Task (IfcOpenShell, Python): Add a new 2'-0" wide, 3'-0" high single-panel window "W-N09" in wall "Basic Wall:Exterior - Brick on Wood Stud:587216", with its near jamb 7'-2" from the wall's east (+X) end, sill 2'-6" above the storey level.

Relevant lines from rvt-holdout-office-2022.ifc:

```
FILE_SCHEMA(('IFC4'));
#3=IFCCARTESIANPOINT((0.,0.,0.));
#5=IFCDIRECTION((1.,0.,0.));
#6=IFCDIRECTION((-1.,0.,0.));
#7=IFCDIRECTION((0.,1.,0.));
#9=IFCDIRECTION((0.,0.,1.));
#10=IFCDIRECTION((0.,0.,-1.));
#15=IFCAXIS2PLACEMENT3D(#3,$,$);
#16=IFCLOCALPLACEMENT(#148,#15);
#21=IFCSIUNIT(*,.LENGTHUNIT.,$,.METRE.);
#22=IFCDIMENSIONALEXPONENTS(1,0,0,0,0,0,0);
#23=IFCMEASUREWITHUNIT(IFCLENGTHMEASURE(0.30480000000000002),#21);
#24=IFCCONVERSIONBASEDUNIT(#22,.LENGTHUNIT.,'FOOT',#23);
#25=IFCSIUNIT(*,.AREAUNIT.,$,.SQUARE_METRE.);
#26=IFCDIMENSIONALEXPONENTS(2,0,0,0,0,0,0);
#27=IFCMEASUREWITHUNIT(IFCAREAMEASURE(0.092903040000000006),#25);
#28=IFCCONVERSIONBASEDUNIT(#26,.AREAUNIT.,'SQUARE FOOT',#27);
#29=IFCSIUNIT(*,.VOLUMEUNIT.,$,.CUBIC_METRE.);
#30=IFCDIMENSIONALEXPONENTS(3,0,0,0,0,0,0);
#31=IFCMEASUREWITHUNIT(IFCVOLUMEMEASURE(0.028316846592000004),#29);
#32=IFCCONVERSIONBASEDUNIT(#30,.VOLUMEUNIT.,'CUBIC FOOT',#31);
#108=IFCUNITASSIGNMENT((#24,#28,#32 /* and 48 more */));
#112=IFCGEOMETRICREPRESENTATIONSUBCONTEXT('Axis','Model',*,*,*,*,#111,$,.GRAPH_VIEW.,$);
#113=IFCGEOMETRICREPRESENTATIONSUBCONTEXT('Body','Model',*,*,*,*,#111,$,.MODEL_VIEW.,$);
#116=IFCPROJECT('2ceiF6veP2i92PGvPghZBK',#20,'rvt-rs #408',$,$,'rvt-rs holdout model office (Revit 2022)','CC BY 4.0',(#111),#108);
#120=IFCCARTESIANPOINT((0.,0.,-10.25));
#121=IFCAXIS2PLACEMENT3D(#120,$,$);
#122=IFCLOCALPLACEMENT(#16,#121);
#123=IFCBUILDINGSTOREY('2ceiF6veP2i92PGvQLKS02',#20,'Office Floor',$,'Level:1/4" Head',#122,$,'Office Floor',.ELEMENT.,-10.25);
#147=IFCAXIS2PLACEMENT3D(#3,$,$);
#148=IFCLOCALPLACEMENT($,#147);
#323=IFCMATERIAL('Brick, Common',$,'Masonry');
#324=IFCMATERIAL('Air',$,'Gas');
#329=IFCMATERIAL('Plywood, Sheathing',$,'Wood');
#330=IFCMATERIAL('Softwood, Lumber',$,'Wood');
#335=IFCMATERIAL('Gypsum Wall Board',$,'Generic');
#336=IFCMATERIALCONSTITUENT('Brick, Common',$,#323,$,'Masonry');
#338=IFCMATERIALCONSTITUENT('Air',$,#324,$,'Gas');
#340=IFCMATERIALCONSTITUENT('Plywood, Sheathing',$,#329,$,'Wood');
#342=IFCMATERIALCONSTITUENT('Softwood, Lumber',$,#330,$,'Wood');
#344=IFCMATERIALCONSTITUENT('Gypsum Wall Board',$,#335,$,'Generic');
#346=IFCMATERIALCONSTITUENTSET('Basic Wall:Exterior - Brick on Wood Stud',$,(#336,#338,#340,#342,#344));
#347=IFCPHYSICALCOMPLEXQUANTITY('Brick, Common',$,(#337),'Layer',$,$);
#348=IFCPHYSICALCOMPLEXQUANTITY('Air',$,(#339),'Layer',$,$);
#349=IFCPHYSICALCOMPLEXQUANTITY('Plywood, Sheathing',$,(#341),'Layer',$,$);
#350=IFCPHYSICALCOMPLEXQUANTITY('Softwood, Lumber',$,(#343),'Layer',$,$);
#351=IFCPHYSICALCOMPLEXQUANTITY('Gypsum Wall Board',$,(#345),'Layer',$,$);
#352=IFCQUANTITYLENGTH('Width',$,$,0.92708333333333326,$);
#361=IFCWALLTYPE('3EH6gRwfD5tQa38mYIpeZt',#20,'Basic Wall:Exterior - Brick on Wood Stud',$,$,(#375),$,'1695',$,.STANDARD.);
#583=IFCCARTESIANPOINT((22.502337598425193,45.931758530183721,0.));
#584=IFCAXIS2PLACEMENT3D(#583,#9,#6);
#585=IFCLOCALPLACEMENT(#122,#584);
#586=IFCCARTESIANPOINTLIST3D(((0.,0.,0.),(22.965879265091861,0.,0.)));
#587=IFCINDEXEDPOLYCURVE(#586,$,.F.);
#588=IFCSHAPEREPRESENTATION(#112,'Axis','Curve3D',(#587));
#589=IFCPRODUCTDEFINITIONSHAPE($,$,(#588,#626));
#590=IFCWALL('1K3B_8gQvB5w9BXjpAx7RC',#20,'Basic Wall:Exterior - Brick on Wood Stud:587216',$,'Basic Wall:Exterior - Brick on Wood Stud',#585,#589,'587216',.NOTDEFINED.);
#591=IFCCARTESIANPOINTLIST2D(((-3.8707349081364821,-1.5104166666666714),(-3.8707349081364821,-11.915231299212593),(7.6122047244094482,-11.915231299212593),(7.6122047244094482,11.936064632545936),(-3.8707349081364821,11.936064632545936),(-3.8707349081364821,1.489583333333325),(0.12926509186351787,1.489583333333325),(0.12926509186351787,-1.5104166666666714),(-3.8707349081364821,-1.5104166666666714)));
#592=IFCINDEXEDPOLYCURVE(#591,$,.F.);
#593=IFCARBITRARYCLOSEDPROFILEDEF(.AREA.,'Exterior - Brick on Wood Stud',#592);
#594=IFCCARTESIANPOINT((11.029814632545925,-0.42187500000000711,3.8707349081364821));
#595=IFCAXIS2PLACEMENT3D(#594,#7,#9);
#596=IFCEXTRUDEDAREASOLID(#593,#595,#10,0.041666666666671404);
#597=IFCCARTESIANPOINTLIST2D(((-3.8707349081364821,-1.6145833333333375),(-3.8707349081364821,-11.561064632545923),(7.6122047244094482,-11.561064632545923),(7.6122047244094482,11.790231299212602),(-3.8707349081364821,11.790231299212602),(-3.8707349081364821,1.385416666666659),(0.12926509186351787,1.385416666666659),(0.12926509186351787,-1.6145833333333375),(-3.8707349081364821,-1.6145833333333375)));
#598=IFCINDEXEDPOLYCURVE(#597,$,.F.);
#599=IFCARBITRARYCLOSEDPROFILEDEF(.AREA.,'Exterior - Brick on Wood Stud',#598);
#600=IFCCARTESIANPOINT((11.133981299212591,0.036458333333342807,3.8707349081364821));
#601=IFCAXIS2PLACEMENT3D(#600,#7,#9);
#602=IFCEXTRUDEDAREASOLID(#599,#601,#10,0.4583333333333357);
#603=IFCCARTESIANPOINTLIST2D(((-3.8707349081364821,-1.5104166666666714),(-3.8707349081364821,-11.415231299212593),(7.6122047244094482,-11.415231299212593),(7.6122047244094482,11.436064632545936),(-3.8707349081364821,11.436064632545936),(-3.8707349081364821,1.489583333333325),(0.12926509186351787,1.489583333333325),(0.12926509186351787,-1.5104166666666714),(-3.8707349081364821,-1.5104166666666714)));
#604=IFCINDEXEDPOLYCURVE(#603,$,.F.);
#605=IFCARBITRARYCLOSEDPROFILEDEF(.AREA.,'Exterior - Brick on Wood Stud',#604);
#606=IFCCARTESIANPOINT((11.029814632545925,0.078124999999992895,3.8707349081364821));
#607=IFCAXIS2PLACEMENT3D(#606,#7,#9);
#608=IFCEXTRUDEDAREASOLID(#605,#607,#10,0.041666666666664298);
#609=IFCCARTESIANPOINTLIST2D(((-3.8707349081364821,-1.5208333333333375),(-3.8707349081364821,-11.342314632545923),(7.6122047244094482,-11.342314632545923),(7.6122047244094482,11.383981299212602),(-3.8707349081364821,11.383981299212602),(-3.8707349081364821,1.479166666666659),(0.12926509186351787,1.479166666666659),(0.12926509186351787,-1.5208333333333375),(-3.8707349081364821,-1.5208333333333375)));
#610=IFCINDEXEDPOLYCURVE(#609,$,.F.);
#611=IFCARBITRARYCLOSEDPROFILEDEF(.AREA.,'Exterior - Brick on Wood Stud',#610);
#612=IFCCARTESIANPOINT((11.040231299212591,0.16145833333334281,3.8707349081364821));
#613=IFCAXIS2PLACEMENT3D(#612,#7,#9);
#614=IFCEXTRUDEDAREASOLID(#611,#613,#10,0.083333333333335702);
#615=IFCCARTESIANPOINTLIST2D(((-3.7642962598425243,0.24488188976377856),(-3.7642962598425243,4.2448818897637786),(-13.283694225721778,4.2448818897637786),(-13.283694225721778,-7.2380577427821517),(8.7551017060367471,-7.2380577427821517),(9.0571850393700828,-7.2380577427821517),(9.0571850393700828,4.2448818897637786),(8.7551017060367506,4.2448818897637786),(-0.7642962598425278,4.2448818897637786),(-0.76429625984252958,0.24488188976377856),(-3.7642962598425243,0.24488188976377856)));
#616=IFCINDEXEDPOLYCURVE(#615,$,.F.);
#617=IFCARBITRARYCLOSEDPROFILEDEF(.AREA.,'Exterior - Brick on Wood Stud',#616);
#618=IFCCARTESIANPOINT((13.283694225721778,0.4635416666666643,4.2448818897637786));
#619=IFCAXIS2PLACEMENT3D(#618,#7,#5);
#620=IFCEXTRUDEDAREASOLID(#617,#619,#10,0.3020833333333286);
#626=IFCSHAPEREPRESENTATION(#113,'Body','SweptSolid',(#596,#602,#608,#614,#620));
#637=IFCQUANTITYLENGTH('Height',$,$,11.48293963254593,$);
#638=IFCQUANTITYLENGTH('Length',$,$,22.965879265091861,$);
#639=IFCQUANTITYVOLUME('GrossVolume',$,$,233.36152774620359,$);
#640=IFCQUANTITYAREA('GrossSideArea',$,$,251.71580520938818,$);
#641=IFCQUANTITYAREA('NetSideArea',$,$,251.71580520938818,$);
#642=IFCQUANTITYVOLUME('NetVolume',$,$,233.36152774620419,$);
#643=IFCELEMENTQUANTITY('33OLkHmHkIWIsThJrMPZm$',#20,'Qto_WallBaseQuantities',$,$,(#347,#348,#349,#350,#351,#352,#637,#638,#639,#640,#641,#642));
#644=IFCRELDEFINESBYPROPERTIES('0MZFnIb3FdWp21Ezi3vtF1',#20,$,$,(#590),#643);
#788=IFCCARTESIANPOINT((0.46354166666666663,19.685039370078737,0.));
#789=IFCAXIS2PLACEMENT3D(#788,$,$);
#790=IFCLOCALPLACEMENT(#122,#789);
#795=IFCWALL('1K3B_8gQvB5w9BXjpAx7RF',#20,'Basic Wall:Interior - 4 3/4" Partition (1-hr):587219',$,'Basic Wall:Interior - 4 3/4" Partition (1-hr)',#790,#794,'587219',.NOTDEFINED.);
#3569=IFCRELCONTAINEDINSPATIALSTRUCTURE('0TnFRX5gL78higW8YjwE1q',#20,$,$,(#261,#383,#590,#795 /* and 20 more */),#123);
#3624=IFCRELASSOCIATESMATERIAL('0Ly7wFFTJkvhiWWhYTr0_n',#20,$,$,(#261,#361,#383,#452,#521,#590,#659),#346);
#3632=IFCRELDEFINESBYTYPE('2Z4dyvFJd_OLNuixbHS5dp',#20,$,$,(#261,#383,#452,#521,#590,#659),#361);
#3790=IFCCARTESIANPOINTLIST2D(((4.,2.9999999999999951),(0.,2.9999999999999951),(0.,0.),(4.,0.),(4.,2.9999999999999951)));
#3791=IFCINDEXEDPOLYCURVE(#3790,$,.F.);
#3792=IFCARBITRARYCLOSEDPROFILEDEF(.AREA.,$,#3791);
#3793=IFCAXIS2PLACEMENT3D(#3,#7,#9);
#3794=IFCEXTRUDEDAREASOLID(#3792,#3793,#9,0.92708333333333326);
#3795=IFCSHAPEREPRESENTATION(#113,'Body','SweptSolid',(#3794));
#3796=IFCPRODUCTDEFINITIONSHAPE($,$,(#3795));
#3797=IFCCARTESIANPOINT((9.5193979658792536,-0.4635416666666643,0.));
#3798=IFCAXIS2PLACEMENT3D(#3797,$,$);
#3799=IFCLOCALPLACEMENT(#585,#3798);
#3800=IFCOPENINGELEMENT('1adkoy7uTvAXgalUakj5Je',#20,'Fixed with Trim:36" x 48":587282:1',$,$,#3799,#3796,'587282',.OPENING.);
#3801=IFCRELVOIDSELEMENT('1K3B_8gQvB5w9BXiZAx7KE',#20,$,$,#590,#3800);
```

```python
import numpy as np
import ifcopenshell
import ifcopenshell.api.feature
import ifcopenshell.api.geometry
import ifcopenshell.api.pset
import ifcopenshell.api.root
import ifcopenshell.api.spatial
import ifcopenshell.geom
import ifcopenshell.util.element
import ifcopenshell.util.placement
import ifcopenshell.util.representation
import ifcopenshell.util.shape
import ifcopenshell.util.unit

model = ifcopenshell.open("rvt-holdout-office-2022.ifc")
unit_scale = ifcopenshell.util.unit.calculate_unit_scale(model)
area_scale = ifcopenshell.util.unit.calculate_unit_scale(model, "AREAUNIT")
volume_scale = ifcopenshell.util.unit.calculate_unit_scale(model, "VOLUMEUNIT")
settings = ifcopenshell.geom.settings()


def volume(element):
    """Net volume in cubic metres, openings subtracted."""
    shape = ifcopenshell.geom.create_shape(settings, element)
    return ifcopenshell.util.shape.get_volume(shape.geometry)


wall = model.by_guid("1K3B_8gQvB5w9BXjpAx7RC")
storey = ifcopenshell.util.element.get_container(wall, ifc_class="IfcBuildingStorey")
context = ifcopenshell.util.representation.get_context(model, "Model", "Body", "MODEL_VIEW")
before = volume(wall)

width, height, from_end, sill = 0.6096, 0.9144, 2.1844, 0.762  # metres

# The wall runs along its own X axis, and the end named is its -X end.
wall_shape = ifcopenshell.geom.create_shape(settings, wall)
x, y, z = ifcopenshell.util.shape.get_vertices(wall_shape.geometry).T
start = x.min() + from_end
face, thickness = float(y.min()), float(y.max() - y.min())
wall_matrix = ifcopenshell.util.placement.get_local_placement(wall.ObjectPlacement)
level = ifcopenshell.util.placement.get_local_placement(storey.ObjectPlacement)[2, 3]


def in_wall(x, y):
    """Placement at x, y metres in the wall's axes, at sill height."""
    matrix = wall_matrix.copy()
    matrix[:, 3] = wall_matrix @ np.array([x / unit_scale, y / unit_scale, 0.0, 1.0])
    matrix[2, 3] = level + sill / unit_scale
    return matrix


# Opening: a box that overshoots both wall faces by 50 mm.
opening = ifcopenshell.api.root.create_entity(model, ifc_class="IfcOpeningElement", predefined_type="OPENING")
box = ifcopenshell.api.geometry.add_wall_representation(
    model, context=context, length=width, height=height, thickness=thickness + 0.1
)
ifcopenshell.api.geometry.assign_representation(model, product=opening, representation=box)
ifcopenshell.api.geometry.edit_object_placement(model, product=opening, matrix=in_wall(start, face - 0.05), is_si=False)
ifcopenshell.api.feature.add_feature(model, feature=opening, element=wall)

window = ifcopenshell.api.root.create_entity(model, ifc_class="IfcWindow", name="W-N09", predefined_type="WINDOW")
window.OverallWidth, window.OverallHeight = width / unit_scale, height / unit_scale
window.PartitioningType = "SINGLE_PANEL"
body = ifcopenshell.api.geometry.add_window_representation(
    model,
    context=context,
    overall_width=window.OverallWidth,
    overall_height=window.OverallHeight,
    partition_type="SINGLE_PANEL",
)
ifcopenshell.api.geometry.assign_representation(model, product=window, representation=body)
ifcopenshell.api.spatial.assign_container(model, products=[window], relating_structure=storey)
ifcopenshell.api.feature.add_filling(model, opening=opening, element=window)

# Centre the window in the wall's thickness.
ifcopenshell.api.geometry.edit_object_placement(model, product=window, matrix=in_wall(start, face), is_si=False)
window_shape = ifcopenshell.geom.create_shape(settings, window)
depth = ifcopenshell.util.shape.get_vertices(window_shape.geometry)[:, 1]
offset = face + thickness / 2 - (depth.min() + depth.max()) / 2
ifcopenshell.api.geometry.edit_object_placement(model, product=window, matrix=in_wall(start, offset), is_si=False)

after = volume(wall)

# Update the wall's stored quantities.
qto = model.by_id(ifcopenshell.util.element.get_pset(wall, "Qto_WallBaseQuantities", should_inherit=False)["id"])
ifcopenshell.api.pset.edit_qto(model, qto=qto, properties={
    "NetSideArea": after / thickness / area_scale,
    "NetVolume": after / volume_scale,
})

print(f"wall volume {before:.3f} -> {after:.3f} m3")

model.write("rvt-holdout-office-2022_rev.ifc")
```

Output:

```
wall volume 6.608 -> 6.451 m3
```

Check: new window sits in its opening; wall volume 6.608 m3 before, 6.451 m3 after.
